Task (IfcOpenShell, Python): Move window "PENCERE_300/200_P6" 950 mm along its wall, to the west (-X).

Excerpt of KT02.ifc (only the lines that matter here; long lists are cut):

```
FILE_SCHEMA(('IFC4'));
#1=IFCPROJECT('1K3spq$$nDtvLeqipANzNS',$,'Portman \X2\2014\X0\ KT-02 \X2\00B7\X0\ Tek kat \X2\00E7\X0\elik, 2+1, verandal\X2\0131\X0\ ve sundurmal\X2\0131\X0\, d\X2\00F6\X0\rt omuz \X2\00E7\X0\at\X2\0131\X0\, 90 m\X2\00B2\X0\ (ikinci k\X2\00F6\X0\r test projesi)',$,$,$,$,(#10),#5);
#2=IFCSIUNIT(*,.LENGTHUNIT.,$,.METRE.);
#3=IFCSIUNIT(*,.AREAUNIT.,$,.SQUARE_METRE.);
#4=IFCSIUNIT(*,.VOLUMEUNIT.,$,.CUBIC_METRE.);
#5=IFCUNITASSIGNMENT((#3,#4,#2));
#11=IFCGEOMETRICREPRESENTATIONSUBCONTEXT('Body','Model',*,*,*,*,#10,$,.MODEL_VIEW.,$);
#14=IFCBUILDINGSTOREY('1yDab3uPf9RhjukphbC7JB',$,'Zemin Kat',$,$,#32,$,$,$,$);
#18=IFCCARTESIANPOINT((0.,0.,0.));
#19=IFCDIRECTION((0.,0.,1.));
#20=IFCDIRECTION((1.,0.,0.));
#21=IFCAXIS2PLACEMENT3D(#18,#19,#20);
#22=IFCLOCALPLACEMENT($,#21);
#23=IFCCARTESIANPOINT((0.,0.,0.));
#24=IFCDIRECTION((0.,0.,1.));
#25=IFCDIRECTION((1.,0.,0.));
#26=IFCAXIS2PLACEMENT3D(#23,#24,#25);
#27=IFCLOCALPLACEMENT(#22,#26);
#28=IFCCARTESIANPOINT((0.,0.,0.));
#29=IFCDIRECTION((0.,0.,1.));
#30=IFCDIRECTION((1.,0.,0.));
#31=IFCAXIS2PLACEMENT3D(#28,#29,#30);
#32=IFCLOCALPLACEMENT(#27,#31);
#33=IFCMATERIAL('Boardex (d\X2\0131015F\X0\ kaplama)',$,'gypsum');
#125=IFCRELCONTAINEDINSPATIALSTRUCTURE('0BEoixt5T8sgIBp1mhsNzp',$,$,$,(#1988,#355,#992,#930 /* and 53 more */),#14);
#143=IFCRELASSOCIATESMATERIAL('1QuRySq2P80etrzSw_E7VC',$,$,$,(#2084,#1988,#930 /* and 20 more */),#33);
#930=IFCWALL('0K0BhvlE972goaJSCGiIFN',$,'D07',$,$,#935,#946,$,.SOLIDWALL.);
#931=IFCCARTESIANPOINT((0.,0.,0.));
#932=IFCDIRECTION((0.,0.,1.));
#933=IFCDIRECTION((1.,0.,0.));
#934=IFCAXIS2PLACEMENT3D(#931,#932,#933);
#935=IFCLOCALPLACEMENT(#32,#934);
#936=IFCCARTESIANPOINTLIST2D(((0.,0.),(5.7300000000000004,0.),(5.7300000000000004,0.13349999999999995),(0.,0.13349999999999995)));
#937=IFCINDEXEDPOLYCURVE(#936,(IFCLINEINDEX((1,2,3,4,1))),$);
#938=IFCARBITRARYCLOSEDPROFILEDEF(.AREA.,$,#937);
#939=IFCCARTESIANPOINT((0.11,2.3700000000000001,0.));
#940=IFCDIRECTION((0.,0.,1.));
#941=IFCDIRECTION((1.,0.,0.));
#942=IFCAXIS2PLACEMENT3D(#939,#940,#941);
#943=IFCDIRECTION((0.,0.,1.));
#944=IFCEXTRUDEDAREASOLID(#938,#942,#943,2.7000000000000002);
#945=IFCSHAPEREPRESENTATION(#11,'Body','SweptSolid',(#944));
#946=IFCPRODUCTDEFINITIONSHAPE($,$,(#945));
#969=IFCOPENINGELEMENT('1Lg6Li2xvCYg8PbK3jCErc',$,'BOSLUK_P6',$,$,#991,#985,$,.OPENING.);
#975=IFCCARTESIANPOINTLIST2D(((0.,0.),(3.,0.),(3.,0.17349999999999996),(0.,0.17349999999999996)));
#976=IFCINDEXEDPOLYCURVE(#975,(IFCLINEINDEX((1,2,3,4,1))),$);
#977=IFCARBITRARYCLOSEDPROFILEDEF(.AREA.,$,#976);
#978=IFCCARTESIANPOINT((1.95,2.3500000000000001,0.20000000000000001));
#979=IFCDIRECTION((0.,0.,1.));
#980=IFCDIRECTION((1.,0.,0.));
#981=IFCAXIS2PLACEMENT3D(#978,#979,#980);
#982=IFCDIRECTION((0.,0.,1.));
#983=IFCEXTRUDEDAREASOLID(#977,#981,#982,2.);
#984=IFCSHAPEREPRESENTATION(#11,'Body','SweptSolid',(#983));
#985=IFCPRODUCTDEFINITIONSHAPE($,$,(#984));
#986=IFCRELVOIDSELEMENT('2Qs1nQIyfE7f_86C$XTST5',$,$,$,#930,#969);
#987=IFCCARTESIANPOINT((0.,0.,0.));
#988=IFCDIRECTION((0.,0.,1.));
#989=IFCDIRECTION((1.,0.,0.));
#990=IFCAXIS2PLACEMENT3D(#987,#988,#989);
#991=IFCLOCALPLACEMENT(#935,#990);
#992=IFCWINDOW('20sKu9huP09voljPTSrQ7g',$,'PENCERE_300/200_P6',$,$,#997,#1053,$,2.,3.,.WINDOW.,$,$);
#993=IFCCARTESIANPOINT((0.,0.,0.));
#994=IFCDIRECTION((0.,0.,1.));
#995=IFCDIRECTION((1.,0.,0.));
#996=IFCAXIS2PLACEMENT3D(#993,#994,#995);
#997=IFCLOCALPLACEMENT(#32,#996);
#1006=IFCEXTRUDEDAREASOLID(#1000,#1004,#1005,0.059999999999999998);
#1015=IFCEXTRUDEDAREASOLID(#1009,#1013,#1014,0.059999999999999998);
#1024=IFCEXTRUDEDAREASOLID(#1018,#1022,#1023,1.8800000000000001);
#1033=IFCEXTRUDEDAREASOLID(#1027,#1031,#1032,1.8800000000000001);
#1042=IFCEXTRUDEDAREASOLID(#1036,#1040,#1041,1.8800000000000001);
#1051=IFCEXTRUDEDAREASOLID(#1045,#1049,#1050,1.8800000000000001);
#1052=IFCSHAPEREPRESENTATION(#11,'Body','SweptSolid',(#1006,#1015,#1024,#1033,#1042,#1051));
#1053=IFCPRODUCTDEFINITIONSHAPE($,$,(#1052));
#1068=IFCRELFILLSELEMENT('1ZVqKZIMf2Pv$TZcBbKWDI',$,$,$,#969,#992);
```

```python
import ifcopenshell
import ifcopenshell.api.geometry
import ifcopenshell.util.placement
import ifcopenshell.util.unit

model = ifcopenshell.open("KT02.ifc")
unit_scale = ifcopenshell.util.unit.calculate_unit_scale(model)

window = model.by_guid("20sKu9huP09voljPTSrQ7g")
opening = window.FillsVoids[0].RelatingOpeningElement
wall = opening.VoidsElements[0].RelatingBuildingElement

wall_matrix = ifcopenshell.util.placement.get_local_placement(wall.ObjectPlacement)
shift = wall_matrix[:3, 0] * -0.95 / unit_scale
before = ifcopenshell.util.placement.get_local_placement(window.ObjectPlacement)[:3, 3].copy()

# The window is not placed relative to its opening, so move both.
for product in (opening, window):
    matrix = ifcopenshell.util.placement.get_local_placement(product.ObjectPlacement)
    matrix[:3, 3] += shift
    ifcopenshell.api.geometry.edit_object_placement(model, product=product, matrix=matrix, is_si=False)

after = ifcopenshell.util.placement.get_local_placement(window.ObjectPlacement)[:3, 3]
print("window moved by", (after - before).round(3) + 0.0)

model.write("KT02_updated.ifc")
```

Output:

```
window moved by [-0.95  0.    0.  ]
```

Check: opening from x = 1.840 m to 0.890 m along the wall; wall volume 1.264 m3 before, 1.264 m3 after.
